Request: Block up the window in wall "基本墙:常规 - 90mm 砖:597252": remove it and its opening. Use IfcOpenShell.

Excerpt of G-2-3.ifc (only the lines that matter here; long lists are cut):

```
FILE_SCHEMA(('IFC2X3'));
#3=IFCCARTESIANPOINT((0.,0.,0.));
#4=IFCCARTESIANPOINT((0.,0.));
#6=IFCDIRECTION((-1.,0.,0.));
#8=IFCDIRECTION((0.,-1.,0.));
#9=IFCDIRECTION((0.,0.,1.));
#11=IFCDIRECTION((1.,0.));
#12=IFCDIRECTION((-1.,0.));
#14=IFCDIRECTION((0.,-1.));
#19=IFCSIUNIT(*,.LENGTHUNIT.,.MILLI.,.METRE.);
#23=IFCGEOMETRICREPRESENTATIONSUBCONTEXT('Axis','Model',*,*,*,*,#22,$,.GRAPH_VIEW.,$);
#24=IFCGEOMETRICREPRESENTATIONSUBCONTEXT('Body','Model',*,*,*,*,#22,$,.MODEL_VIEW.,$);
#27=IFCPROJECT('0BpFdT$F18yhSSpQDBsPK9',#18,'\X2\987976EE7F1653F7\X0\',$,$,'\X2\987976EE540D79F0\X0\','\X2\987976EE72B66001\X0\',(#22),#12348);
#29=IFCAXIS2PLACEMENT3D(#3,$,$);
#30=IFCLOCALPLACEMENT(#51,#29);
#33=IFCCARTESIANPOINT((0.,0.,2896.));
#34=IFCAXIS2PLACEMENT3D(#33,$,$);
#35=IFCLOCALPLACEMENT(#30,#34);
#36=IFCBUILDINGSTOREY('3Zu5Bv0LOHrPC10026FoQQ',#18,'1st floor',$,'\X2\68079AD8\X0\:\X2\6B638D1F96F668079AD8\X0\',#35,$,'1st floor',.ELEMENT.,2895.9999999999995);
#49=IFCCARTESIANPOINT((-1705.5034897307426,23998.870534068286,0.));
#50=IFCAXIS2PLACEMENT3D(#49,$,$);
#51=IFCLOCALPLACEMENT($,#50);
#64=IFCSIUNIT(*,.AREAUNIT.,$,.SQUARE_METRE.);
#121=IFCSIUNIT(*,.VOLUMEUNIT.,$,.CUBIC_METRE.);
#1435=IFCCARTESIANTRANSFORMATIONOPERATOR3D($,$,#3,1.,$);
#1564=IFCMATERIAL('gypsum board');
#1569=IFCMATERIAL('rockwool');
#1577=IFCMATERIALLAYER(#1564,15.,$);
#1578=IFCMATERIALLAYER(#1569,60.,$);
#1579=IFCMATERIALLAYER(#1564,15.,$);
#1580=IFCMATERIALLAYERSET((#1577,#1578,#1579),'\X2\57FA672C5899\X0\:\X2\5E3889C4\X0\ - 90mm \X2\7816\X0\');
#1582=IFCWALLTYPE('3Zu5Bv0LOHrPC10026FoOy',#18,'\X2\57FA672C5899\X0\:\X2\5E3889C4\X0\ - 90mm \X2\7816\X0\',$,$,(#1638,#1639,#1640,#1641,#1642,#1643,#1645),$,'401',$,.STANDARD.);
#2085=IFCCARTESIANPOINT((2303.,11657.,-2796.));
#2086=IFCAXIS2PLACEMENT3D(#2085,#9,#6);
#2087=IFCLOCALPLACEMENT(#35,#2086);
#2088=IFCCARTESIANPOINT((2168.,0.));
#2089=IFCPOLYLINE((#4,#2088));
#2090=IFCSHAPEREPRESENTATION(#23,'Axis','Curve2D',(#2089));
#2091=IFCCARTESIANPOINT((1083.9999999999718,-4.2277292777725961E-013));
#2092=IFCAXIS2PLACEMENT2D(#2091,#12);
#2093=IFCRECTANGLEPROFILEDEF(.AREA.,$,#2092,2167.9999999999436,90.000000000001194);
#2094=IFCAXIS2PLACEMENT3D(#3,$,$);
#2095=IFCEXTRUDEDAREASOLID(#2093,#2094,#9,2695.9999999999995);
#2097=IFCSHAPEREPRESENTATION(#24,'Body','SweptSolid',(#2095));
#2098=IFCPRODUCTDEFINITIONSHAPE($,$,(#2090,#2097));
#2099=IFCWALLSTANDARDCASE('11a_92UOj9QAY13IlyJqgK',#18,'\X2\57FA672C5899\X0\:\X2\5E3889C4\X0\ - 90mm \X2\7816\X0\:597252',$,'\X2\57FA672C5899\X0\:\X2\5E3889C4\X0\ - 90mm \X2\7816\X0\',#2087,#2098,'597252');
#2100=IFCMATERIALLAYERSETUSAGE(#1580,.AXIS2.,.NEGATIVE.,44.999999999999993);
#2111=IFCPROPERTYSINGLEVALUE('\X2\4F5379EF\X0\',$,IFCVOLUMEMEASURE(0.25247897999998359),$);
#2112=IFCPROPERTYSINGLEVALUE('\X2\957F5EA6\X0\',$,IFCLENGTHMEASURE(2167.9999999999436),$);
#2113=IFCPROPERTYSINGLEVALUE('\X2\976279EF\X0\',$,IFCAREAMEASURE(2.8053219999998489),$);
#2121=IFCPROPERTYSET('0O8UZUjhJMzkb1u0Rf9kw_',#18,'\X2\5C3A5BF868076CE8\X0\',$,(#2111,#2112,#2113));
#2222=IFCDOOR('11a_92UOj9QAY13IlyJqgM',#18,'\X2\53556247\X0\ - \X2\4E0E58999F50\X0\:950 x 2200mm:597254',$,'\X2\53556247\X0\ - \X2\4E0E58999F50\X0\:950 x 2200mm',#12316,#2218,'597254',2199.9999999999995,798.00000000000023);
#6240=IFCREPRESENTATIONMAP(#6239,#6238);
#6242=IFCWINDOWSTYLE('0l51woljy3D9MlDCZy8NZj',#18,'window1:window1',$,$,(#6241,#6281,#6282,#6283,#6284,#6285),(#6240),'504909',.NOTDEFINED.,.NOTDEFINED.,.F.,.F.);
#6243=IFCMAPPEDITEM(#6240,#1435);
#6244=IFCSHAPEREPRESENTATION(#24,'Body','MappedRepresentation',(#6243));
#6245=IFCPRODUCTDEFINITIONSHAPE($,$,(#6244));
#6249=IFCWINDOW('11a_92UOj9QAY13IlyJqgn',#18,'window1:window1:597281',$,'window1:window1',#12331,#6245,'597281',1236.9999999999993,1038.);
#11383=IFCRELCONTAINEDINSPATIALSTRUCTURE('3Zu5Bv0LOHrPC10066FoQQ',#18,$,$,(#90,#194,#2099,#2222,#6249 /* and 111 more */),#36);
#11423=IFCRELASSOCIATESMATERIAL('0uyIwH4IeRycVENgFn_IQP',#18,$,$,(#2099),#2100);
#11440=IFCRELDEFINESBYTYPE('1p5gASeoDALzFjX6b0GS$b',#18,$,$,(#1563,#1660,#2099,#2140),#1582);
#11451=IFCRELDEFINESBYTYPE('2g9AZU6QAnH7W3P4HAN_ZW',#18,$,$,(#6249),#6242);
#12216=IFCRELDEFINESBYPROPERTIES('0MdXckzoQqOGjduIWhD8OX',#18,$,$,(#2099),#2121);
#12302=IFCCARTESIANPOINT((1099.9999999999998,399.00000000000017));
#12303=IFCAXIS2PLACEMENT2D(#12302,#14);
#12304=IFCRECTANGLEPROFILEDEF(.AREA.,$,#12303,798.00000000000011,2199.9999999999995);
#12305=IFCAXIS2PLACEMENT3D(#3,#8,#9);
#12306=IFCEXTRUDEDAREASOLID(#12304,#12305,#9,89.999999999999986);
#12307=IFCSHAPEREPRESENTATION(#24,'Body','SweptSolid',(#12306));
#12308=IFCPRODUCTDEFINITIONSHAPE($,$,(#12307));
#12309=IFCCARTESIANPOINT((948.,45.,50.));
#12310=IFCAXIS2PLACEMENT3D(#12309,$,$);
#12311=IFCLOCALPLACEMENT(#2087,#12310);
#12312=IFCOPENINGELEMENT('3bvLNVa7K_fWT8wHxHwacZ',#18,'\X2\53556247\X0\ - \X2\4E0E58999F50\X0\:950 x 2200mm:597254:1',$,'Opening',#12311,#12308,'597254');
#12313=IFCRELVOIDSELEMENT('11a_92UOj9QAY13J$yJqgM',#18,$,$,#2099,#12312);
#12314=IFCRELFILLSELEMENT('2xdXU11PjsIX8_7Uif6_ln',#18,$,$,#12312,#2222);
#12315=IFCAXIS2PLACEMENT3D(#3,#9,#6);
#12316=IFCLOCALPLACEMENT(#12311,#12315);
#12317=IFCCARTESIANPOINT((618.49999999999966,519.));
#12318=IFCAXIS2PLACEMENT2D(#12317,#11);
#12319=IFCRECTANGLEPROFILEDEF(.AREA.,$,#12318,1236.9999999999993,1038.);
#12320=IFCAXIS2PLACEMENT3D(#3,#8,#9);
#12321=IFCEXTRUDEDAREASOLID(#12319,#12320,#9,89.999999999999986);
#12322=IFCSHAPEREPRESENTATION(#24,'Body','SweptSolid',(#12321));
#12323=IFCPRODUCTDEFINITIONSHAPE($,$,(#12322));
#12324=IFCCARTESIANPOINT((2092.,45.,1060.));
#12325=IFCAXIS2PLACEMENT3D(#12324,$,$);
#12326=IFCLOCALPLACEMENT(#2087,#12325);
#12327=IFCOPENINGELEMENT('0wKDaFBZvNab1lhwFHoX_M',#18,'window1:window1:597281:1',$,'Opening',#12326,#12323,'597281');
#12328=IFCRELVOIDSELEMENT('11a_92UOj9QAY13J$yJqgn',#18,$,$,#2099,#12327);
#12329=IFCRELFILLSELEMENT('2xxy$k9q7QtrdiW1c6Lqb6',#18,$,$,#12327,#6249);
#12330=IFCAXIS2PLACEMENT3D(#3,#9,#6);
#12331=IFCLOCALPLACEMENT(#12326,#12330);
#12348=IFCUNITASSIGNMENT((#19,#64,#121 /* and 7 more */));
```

```python
import ifcopenshell
import ifcopenshell.api.feature
import ifcopenshell.api.pset
import ifcopenshell.api.root
import ifcopenshell.geom
import ifcopenshell.util.element
import ifcopenshell.util.shape
import ifcopenshell.util.unit

model = ifcopenshell.open("G-2-3.ifc")
area_scale = ifcopenshell.util.unit.calculate_unit_scale(model, "AREAUNIT")
volume_scale = ifcopenshell.util.unit.calculate_unit_scale(model, "VOLUMEUNIT")
settings = ifcopenshell.geom.settings()


def volume(element):
    """Net volume in cubic metres, openings subtracted."""
    shape = ifcopenshell.geom.create_shape(settings, element)
    return ifcopenshell.util.shape.get_volume(shape.geometry)


window = model.by_guid("11a_92UOj9QAY13IlyJqgn")
opening = window.FillsVoids[0].RelatingOpeningElement
wall = opening.VoidsElements[0].RelatingBuildingElement
before = volume(wall)

ifcopenshell.api.root.remove_product(model, product=window)
ifcopenshell.api.feature.remove_feature(model, feature=opening)

after = volume(wall)
thickness = 0.09  # wall thickness in metres

# Update the wall's stored quantities.
pset = model.by_id(ifcopenshell.util.element.get_pset(wall, "尺寸标注", should_inherit=False)["id"])
ifcopenshell.api.pset.edit_pset(model, pset=pset, properties={
    "体积": model.create_entity("IfcVolumeMeasure", after / volume_scale),
    "面积": model.create_entity("IfcAreaMeasure", after / thickness / area_scale),
})

print(f"wall volume {before:.3f} -> {after:.3f} m3")

model.write("G-2-3_rev.ifc")
```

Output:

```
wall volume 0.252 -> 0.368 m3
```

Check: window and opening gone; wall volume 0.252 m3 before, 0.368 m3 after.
